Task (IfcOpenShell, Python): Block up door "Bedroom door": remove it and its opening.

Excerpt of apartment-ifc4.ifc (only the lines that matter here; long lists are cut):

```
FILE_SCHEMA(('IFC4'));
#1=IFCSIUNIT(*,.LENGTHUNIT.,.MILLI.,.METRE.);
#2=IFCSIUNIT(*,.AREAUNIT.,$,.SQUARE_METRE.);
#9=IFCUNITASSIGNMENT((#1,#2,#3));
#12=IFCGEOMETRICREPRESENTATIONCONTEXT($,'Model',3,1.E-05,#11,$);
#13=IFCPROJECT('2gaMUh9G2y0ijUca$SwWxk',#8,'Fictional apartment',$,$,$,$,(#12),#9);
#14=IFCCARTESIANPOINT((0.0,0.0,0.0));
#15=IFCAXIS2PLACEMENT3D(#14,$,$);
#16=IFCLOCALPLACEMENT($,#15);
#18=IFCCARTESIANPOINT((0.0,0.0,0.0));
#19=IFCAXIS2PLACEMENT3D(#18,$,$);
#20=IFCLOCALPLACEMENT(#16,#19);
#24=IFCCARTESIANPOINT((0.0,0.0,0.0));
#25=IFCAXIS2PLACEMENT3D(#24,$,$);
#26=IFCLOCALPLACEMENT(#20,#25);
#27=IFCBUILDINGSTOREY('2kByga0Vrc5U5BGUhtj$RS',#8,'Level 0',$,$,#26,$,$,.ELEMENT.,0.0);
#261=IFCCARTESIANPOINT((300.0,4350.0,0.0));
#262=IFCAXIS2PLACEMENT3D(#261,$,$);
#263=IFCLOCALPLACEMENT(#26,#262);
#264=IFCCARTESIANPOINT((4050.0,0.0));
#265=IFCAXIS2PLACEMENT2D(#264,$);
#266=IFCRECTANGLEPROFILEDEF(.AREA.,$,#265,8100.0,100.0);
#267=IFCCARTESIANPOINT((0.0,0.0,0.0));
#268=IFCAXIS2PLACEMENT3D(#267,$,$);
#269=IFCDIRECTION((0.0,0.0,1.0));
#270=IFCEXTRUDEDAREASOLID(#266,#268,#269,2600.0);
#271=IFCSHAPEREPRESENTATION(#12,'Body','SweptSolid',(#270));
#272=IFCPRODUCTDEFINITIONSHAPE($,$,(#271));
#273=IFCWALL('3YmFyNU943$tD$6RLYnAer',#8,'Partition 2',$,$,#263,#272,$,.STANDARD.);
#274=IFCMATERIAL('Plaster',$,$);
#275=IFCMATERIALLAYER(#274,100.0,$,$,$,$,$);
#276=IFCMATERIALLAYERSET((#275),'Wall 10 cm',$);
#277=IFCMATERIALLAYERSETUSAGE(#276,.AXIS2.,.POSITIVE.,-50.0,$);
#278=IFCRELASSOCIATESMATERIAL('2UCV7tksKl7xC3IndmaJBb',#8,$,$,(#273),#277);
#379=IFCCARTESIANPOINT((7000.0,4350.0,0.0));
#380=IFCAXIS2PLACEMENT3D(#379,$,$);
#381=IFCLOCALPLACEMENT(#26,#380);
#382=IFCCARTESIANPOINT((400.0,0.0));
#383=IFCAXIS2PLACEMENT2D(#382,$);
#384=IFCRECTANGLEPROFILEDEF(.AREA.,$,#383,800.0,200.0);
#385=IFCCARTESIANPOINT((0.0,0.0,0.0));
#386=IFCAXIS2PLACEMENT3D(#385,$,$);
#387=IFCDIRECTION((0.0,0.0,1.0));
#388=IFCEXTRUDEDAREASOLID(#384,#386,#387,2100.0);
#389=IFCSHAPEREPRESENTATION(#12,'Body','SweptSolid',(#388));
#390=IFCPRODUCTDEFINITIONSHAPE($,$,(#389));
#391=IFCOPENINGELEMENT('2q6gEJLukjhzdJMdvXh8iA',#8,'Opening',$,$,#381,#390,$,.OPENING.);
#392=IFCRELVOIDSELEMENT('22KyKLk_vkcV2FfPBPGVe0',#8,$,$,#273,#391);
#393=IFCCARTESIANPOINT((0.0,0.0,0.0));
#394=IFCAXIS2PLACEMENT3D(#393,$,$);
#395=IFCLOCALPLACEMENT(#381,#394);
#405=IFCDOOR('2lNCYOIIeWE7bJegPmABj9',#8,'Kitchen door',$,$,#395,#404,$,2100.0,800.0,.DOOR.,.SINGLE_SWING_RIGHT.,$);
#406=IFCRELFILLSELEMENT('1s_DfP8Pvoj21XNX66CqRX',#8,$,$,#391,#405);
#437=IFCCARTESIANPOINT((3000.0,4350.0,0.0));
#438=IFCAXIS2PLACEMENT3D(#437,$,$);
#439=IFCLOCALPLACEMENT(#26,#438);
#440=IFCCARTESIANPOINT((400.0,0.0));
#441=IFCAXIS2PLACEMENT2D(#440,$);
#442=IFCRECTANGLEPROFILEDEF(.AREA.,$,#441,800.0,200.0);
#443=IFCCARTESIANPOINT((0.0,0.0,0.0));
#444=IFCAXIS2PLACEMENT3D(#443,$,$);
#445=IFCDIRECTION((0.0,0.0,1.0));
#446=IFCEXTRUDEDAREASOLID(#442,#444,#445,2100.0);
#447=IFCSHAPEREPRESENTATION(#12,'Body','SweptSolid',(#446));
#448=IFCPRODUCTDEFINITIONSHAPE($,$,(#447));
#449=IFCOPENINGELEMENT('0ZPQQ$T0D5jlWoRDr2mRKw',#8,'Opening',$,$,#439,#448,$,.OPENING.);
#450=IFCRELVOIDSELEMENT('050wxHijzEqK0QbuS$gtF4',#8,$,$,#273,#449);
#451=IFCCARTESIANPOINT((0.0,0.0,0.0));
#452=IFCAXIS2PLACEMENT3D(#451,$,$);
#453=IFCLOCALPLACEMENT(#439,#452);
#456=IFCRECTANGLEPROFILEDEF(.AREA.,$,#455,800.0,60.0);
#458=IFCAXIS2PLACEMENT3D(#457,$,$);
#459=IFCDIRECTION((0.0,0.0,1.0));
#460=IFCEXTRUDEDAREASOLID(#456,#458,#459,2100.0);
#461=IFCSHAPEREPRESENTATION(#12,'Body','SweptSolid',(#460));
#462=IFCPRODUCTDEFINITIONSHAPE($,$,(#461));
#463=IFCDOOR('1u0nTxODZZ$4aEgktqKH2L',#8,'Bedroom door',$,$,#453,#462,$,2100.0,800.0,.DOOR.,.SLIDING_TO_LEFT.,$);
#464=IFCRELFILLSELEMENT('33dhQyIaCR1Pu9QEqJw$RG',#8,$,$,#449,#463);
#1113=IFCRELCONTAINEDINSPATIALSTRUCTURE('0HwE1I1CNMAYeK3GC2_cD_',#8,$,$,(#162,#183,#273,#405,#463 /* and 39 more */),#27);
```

```python
import ifcopenshell
import ifcopenshell.api.feature
import ifcopenshell.api.root
import ifcopenshell.geom
import ifcopenshell.util.shape

model = ifcopenshell.open("apartment-ifc4.ifc")
settings = ifcopenshell.geom.settings()


def volume(element):
    """Net volume in cubic metres, openings subtracted."""
    shape = ifcopenshell.geom.create_shape(settings, element)
    return ifcopenshell.util.shape.get_volume(shape.geometry)


door = model.by_guid("1u0nTxODZZ$4aEgktqKH2L")
opening = door.FillsVoids[0].RelatingOpeningElement
wall = opening.VoidsElements[0].RelatingBuildingElement
before = volume(wall)

ifcopenshell.api.root.remove_product(model, product=door)
ifcopenshell.api.feature.remove_feature(model, feature=opening)

after = volume(wall)

print(f"wall volume {before:.3f} -> {after:.3f} m3")

model.write("apartment-ifc4-out.ifc")
```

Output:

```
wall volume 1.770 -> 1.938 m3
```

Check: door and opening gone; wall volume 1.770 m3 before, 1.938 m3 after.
